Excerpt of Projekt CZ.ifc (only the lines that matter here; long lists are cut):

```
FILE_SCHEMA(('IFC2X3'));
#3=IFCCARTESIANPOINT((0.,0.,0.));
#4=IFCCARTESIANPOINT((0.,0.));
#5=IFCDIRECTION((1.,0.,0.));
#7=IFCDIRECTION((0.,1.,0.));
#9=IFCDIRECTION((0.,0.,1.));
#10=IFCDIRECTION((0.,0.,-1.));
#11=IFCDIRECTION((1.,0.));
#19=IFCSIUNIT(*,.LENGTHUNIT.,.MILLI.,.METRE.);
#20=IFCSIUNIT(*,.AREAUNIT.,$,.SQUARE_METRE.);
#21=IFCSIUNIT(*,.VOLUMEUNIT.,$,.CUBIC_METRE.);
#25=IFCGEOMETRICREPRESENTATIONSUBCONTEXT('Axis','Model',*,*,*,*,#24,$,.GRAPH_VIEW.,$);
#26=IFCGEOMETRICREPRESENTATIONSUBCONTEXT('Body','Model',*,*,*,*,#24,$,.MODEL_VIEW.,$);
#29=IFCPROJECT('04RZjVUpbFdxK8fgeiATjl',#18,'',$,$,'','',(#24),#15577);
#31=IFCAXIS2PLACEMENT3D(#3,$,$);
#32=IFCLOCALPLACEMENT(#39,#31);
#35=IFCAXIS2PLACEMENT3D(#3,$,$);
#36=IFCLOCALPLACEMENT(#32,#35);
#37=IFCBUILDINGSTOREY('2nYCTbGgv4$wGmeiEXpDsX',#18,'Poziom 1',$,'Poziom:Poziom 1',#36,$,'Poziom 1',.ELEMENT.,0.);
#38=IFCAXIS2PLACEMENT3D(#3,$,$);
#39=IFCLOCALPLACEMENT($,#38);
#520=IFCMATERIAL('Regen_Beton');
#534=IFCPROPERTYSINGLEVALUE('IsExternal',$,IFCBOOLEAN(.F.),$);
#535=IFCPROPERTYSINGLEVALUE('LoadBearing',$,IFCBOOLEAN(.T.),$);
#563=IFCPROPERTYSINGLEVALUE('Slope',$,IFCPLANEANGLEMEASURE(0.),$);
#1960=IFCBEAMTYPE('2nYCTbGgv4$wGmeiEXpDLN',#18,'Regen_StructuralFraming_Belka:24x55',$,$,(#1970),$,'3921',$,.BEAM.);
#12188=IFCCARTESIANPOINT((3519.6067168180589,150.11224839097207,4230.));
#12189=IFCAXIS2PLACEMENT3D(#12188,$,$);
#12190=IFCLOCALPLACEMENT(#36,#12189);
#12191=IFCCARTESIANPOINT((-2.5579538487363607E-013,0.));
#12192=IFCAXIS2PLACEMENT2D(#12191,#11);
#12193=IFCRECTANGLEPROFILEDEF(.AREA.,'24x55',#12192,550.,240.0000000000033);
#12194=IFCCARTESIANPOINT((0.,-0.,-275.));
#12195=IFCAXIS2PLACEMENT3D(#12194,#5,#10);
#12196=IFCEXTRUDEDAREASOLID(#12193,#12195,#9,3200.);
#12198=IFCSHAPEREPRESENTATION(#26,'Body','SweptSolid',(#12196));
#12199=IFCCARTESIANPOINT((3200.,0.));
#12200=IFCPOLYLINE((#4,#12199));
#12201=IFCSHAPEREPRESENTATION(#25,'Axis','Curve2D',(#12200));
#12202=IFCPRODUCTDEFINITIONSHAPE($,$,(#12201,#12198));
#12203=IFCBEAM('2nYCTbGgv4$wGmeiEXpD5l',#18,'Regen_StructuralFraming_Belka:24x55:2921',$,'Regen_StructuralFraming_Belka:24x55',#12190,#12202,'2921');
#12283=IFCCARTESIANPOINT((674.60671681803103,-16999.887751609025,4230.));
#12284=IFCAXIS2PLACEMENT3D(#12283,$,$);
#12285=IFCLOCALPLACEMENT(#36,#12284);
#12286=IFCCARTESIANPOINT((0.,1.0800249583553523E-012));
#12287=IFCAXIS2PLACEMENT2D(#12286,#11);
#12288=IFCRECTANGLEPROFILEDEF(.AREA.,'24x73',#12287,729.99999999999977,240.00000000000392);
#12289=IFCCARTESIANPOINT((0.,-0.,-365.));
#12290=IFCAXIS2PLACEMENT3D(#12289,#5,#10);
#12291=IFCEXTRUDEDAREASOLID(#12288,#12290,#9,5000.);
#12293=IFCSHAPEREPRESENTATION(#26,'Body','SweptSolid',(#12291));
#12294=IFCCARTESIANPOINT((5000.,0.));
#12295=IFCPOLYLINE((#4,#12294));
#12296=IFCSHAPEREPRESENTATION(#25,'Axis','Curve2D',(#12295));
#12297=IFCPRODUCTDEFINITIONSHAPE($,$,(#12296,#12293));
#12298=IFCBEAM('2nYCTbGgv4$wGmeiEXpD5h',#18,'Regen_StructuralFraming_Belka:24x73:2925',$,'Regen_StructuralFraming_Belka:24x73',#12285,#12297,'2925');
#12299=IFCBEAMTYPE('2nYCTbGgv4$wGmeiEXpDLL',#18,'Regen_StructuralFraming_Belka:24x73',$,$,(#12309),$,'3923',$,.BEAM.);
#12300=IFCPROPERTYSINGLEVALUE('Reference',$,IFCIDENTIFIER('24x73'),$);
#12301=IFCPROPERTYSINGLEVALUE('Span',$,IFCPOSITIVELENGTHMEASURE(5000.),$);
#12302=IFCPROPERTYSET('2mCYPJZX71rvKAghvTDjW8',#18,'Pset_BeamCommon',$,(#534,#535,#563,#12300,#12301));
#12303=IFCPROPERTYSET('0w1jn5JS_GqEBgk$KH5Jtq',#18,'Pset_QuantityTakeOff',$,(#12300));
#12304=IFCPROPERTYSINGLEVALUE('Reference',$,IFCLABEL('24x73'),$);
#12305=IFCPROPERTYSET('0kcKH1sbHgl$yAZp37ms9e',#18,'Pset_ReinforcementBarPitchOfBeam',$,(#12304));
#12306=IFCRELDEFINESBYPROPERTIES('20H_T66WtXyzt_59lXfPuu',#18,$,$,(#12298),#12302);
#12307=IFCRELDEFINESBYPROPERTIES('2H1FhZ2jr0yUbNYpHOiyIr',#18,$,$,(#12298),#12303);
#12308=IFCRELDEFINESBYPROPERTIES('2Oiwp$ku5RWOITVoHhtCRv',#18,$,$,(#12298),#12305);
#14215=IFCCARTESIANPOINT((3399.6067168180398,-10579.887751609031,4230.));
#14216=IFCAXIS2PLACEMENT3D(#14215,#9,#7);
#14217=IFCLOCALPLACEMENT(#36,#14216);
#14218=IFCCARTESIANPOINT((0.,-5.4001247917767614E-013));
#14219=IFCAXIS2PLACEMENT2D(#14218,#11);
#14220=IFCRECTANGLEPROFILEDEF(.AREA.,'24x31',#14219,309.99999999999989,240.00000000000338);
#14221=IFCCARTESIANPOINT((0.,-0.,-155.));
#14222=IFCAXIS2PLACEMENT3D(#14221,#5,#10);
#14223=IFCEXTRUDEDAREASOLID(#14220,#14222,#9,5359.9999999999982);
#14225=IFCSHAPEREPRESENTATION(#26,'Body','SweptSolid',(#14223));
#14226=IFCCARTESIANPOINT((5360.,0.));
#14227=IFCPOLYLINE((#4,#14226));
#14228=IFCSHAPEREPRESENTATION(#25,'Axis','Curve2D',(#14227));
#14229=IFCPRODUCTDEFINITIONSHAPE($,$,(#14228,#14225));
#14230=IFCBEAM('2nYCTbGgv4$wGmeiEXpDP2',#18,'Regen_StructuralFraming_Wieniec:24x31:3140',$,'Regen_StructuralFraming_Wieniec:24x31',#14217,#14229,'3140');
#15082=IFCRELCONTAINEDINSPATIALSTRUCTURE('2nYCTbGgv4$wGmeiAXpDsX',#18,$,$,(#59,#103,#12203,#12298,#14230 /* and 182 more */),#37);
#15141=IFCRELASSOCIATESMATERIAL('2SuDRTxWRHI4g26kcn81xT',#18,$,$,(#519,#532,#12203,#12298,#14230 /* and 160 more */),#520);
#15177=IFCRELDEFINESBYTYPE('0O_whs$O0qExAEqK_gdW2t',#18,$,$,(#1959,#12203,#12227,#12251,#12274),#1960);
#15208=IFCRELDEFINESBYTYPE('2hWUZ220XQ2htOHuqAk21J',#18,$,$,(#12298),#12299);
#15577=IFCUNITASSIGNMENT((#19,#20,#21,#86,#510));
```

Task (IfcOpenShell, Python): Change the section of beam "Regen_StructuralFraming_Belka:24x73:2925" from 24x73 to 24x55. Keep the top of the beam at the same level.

```python
import ifcopenshell
import ifcopenshell.api.pset
import ifcopenshell.api.type
import ifcopenshell.util.element
import ifcopenshell.util.representation

model = ifcopenshell.open("Projekt CZ.ifc")

member = model.by_guid("2nYCTbGgv4$wGmeiEXpD5h")
source = next(p for p in model.by_type("IfcRectangleProfileDef") if p.ProfileName == "24x55")

body = ifcopenshell.util.representation.get_representation(member, "Model", "Body")
solid = body.Items[0]
old_profile = solid.SweptArea

# Copy the section's sizes but keep this member's own profile position.
profile = ifcopenshell.util.element.copy(model, source)
# Profiles are centred, so shift by half the change in depth to hold the top.
shift = (old_profile.XDim - profile.XDim) / 2
x, y = old_profile.Position.Location.Coordinates
up = (-1.0, 0.0)  # upwards, in the solid's own plane
location = model.createIfcCartesianPoint((x + up[0] * shift, y + up[1] * shift))
profile.Position = model.createIfcAxis2Placement2D(location, old_profile.Position.RefDirection)
solid.SweptArea = profile
if not model.get_total_inverses(old_profile):
    ifcopenshell.util.element.remove_deep2(model, old_profile)

new_type = model.by_guid("2nYCTbGgv4$wGmeiEXpDLN")
ifcopenshell.api.type.assign_type(
    model, related_objects=[member], relating_type=new_type, should_map_representations=False
)
member.Name = member.Name.replace("24x73", "24x55")
member.ObjectType = "Regen_StructuralFraming_Belka:24x55"
pset = model.by_id(ifcopenshell.util.element.get_pset(member, "Pset_BeamCommon", should_inherit=False)["id"])
ifcopenshell.api.pset.edit_pset(model, pset=pset, properties={"Reference": "24x55"})
pset = model.by_id(ifcopenshell.util.element.get_pset(member, "Pset_QuantityTakeOff", should_inherit=False)["id"])
ifcopenshell.api.pset.edit_pset(model, pset=pset, properties={"Reference": "24x55"})
pset = model.by_id(ifcopenshell.util.element.get_pset(member, "Pset_ReinforcementBarPitchOfBeam", should_inherit=False)["id"])
ifcopenshell.api.pset.edit_pset(model, pset=pset, properties={"Reference": "24x55"})

print(solid.SweptArea)

model.write("Projekt CZ_edited.ifc")
```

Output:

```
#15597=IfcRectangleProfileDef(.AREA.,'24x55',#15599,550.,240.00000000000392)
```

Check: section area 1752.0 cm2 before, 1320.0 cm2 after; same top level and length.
